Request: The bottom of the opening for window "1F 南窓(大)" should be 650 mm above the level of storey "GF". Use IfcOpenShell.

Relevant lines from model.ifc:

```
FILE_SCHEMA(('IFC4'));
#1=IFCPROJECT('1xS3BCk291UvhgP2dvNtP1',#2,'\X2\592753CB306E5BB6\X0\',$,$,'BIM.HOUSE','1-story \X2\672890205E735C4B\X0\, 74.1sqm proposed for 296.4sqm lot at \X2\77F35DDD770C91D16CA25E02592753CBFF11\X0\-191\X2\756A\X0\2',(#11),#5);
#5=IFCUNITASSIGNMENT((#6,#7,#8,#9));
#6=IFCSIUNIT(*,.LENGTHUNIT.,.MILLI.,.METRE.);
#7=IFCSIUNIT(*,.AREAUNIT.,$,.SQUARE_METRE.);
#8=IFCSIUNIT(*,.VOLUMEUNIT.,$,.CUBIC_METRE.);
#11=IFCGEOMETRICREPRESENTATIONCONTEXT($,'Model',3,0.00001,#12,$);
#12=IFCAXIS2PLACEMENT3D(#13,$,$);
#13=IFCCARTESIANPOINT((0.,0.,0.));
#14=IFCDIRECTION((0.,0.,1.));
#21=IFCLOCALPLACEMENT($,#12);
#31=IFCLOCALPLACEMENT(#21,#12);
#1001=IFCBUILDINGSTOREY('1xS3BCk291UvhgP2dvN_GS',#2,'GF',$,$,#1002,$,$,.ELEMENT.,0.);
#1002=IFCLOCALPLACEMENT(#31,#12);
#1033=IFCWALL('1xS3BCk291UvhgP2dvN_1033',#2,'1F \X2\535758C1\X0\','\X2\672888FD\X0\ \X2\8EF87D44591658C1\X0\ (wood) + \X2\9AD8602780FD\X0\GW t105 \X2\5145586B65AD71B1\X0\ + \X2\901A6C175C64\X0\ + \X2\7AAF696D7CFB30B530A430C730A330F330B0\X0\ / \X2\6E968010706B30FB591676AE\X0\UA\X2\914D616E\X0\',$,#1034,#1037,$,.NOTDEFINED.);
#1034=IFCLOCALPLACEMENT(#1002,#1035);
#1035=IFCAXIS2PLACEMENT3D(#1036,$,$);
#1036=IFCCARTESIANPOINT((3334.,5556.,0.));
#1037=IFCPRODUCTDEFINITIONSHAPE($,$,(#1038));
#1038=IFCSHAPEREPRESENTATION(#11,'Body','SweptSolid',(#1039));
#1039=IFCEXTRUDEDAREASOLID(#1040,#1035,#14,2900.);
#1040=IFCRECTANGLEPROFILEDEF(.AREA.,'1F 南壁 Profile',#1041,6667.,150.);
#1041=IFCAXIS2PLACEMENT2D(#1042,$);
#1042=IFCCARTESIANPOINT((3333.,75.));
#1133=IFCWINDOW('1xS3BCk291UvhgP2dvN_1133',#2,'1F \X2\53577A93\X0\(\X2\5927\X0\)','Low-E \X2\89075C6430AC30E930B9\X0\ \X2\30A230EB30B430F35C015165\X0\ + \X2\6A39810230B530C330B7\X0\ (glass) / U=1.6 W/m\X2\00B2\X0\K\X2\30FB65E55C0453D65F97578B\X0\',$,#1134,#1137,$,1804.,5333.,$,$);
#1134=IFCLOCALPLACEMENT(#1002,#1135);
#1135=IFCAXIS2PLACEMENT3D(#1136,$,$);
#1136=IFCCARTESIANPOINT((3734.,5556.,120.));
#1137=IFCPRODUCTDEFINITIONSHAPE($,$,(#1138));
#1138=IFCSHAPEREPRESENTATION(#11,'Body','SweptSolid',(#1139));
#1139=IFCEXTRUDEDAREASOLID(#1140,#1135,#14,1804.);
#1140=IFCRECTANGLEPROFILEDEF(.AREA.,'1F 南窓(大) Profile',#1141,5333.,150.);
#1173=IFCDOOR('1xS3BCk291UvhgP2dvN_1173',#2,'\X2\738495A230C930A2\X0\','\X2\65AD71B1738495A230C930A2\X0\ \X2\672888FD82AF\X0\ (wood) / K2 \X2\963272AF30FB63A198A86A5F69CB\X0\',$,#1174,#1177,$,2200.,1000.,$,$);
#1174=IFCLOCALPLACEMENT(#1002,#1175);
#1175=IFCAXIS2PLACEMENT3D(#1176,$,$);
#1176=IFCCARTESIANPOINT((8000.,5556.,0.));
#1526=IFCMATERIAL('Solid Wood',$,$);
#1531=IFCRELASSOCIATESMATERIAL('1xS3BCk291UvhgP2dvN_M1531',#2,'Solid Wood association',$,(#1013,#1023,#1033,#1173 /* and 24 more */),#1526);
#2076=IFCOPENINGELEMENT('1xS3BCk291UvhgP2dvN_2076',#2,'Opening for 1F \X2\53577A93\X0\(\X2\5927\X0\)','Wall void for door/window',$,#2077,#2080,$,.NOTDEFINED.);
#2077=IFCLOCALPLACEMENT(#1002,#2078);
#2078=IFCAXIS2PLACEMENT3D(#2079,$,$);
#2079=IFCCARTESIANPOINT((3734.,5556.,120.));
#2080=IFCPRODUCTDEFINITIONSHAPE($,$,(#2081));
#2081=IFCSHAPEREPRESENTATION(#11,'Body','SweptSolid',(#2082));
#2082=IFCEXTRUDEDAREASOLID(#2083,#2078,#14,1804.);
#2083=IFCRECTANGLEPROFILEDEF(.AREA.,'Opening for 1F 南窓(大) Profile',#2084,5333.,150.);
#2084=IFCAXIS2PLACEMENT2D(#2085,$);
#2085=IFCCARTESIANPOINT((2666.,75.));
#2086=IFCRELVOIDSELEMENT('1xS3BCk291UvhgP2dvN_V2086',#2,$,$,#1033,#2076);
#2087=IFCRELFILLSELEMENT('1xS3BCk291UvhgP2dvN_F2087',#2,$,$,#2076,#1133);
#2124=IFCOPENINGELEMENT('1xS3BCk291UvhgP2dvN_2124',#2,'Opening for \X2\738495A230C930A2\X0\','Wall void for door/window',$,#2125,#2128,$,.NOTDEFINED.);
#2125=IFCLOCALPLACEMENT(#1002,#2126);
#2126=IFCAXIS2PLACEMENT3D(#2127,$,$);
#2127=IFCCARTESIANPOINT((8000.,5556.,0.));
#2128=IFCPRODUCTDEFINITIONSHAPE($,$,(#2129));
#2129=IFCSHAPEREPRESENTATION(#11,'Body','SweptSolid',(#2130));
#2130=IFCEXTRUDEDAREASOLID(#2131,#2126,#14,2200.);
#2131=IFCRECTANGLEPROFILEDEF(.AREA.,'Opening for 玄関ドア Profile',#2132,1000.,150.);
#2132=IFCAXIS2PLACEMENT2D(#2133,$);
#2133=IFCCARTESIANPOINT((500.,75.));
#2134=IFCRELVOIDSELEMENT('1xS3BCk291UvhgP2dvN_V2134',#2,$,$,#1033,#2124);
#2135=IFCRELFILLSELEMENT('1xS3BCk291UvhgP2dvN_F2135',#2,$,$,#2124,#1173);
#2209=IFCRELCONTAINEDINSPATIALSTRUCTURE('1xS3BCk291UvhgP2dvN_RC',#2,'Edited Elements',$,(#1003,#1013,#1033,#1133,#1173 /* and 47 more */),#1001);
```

```python
import numpy as np
import ifcopenshell
import ifcopenshell.api.geometry
import ifcopenshell.geom
import ifcopenshell.util.element
import ifcopenshell.util.placement
import ifcopenshell.util.shape
import ifcopenshell.util.unit

model = ifcopenshell.open("model.ifc")
unit_scale = ifcopenshell.util.unit.calculate_unit_scale(model)

window = model.by_guid("1xS3BCk291UvhgP2dvN_1133")
opening = window.FillsVoids[0].RelatingOpeningElement
storey = ifcopenshell.util.element.get_container(window, ifc_class="IfcBuildingStorey")
level = ifcopenshell.util.placement.get_local_placement(storey.ObjectPlacement)[2, 3]

# The opening's origin need not be at the sill, so measure its lowest point.
shape = ifcopenshell.geom.create_shape(ifcopenshell.geom.settings(), opening)
bottom = ifcopenshell.util.shape.get_shape_bottom_elevation(shape, shape.geometry) / unit_scale
dz = level + 0.65 / unit_scale - bottom

shift = np.array([0.0, 0.0, dz])
# The window is not placed relative to its opening, so move both.
for product in (opening, window):
    matrix = ifcopenshell.util.placement.get_local_placement(product.ObjectPlacement)
    matrix[:3, 3] += shift
    ifcopenshell.api.geometry.edit_object_placement(model, product=product, matrix=matrix, is_si=False)

print(f"moved by {dz * unit_scale:+.3f} m")

model.write("model-out.ifc")
```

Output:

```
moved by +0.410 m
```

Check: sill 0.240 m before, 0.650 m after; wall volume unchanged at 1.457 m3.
